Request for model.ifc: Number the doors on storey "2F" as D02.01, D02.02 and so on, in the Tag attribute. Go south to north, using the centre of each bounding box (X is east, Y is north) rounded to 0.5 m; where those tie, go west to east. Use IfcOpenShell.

First a look at what the model holds.

```python
import ifcopenshell
import ifcopenshell.util.element
import ifcopenshell.util.placement

model = ifcopenshell.open("model.ifc")
print(model.schema)
storey = next(s for s in model.by_type("IfcBuildingStorey") if s.Name == "2F")
doors = [e for e in ifcopenshell.util.element.get_decomposition(storey) if e.is_a("IfcDoor")]
for e in sorted(doors, key=lambda e: e.id()):
    origin = ifcopenshell.util.placement.get_local_placement(e.ObjectPlacement)[:3, 3]
    print(e.id(), e.Tag, e.Name, origin.round(2) + 0.0, sep=" | ")
```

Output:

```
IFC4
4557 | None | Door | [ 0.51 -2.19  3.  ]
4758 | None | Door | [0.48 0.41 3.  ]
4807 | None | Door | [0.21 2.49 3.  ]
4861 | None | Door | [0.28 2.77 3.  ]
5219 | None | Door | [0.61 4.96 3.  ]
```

```python
import ifcopenshell
import ifcopenshell.geom
import ifcopenshell.util.element
import ifcopenshell.util.shape

model = ifcopenshell.open("model.ifc")
settings = ifcopenshell.geom.settings()
settings.set("use-world-coords", True)


def centre(element):
    shape = ifcopenshell.geom.create_shape(settings, element)
    return ifcopenshell.util.shape.get_bbox_centroid(shape.geometry)


storey = next(s for s in model.by_type("IfcBuildingStorey") if s.Name == "2F")
doors = [e for e in ifcopenshell.util.element.get_decomposition(storey) if e.is_a("IfcDoor")]

# Insertion points can sit at a corner or the storey origin, so sort by the geometry (in metres).
centres = {e: centre(e) for e in doors}
doors.sort(key=lambda e: (round(centres[e][1] / 0.5), centres[e][0]))

for i, e in enumerate(doors, start=1):
    number = f"D02.{i:02d}"
    e.Tag = number
    print(e.id(), number)

model.write("model_edited.ifc")
```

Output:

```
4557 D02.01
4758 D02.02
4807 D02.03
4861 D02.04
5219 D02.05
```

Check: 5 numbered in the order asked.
